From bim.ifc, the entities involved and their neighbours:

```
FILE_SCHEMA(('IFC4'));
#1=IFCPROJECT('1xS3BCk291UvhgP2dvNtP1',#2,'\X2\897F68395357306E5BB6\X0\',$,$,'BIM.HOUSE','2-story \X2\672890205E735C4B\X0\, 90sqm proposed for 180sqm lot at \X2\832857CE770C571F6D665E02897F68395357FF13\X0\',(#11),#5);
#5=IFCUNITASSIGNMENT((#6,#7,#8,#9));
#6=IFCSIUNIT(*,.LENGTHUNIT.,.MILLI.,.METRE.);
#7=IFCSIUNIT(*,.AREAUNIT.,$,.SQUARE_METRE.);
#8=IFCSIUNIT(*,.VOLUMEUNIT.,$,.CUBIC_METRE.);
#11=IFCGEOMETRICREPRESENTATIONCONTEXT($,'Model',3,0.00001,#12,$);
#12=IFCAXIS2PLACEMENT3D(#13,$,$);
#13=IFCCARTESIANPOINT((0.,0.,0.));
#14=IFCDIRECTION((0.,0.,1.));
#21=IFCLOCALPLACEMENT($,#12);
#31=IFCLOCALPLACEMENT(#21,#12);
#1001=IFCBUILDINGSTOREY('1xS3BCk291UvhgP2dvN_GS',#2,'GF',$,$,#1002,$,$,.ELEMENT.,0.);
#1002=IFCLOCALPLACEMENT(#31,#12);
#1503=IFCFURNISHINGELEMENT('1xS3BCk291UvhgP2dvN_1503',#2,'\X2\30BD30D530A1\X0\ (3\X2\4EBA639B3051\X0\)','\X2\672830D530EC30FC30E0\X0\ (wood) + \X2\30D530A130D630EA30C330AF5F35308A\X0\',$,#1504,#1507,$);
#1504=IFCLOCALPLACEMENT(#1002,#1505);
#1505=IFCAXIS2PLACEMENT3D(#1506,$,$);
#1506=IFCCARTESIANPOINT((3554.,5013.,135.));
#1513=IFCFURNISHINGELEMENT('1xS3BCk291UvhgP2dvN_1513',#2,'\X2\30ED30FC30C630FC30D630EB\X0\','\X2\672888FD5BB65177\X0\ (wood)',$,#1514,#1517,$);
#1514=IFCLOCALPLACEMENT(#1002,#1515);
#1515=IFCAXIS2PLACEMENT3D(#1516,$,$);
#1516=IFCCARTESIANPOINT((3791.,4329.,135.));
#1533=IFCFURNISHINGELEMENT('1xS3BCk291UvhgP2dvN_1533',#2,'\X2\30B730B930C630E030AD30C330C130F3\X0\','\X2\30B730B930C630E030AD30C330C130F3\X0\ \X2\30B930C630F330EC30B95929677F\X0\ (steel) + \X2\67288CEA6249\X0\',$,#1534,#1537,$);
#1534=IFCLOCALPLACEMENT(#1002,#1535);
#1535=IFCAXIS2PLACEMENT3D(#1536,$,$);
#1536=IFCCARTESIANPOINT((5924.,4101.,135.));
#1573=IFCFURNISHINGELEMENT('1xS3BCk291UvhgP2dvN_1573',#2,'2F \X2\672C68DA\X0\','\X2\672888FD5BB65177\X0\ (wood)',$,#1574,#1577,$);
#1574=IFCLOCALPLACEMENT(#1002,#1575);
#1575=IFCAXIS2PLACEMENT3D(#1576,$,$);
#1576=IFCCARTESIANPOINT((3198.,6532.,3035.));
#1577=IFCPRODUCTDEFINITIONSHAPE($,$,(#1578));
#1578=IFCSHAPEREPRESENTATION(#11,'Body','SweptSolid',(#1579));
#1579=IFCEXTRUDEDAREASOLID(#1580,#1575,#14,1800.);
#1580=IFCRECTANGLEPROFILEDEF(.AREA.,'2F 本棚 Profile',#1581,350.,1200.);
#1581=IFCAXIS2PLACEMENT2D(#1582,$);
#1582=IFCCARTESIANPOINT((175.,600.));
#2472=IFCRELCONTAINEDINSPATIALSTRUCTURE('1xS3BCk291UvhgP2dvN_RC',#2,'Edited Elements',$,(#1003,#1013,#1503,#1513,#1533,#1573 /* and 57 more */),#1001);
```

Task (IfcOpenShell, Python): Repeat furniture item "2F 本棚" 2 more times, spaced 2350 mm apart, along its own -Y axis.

```python
import ifcopenshell
import ifcopenshell.api.geometry
import ifcopenshell.api.root
import ifcopenshell.util.element
import ifcopenshell.util.placement

model = ifcopenshell.open("bim.ifc")


def reuse_history(source, copy):
    """copy_class also copies each property set's owner history, people and application; keep the originals."""
    for rel in copy.IsDefinedBy:
        if rel.is_a("IfcRelDefinesByProperties") and (history := rel.RelatingPropertyDefinition.OwnerHistory):
            rel.RelatingPropertyDefinition.OwnerHistory = source.OwnerHistory
            ifcopenshell.util.element.remove_deep2(model, history)


source = model.by_guid("1xS3BCk291UvhgP2dvN_1573")
base = ifcopenshell.util.placement.get_local_placement(source.ObjectPlacement)
step = -base[:3, 1] * 2350.0

for i in range(1, 3):
    copy = ifcopenshell.api.root.copy_class(model, product=source)
    copy.Representation = ifcopenshell.util.element.copy_deep(
        model, source.Representation, exclude=["IfcGeometricRepresentationContext", "IfcRepresentationMap"]
    )
    reuse_history(source, copy)
    matrix = base.copy()
    matrix[:3, 3] += i * step
    print("added at", matrix[:3, 3].round(3) + 0.0)
    ifcopenshell.api.geometry.edit_object_placement(model, product=copy, matrix=matrix, is_si=False)

model.write("bim-out.ifc")
```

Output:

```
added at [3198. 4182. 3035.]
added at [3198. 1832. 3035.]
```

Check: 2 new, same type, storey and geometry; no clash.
